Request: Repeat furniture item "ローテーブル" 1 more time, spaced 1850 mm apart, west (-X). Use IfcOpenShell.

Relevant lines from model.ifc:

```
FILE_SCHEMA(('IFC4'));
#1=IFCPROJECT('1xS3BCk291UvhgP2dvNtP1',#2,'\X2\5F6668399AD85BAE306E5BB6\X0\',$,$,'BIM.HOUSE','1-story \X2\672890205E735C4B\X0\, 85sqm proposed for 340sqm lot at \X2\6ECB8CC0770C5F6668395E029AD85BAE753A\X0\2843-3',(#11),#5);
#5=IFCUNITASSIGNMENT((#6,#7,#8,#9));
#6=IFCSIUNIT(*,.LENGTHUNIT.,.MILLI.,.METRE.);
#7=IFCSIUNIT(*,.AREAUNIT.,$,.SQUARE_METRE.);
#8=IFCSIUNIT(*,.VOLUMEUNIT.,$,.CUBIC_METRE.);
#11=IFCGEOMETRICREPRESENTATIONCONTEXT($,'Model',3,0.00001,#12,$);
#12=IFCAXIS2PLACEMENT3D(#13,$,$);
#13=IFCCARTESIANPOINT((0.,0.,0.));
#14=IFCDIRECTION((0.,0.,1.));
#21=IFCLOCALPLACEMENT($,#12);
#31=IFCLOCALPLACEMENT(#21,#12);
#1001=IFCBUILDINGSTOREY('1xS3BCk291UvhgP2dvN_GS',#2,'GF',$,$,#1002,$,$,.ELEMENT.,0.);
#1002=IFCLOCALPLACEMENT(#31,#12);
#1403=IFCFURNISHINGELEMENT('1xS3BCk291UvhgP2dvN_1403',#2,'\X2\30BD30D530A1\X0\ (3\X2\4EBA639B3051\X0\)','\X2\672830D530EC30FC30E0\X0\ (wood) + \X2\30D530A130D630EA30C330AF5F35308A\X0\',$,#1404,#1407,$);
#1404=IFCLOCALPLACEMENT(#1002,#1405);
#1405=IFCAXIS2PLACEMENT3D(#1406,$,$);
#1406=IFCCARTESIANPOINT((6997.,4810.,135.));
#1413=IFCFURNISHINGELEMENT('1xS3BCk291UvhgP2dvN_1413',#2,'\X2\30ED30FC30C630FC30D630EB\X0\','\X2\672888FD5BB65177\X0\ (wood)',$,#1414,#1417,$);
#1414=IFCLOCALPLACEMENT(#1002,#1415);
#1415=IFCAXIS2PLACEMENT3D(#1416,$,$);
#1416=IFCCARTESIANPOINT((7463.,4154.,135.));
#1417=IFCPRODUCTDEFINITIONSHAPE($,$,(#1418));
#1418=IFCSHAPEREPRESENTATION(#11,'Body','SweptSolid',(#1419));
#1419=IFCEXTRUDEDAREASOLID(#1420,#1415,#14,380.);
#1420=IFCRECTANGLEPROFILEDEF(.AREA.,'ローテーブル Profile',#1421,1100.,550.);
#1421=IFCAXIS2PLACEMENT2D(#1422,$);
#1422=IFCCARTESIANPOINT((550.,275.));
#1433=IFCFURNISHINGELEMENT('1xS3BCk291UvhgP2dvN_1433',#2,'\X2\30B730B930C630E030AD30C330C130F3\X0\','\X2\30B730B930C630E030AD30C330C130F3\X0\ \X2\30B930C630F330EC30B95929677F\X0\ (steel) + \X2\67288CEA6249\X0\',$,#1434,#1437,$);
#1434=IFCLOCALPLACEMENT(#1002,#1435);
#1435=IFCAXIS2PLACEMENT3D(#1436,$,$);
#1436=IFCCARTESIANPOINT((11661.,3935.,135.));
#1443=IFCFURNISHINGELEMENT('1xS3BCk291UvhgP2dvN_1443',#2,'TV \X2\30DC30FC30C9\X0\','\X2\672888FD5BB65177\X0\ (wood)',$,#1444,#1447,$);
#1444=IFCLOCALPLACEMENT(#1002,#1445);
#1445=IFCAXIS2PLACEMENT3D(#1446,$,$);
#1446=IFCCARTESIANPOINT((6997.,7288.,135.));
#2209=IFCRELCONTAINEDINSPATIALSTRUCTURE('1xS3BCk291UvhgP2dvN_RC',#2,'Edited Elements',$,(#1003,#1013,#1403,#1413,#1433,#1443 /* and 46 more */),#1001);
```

```python
import numpy as np
import ifcopenshell
import ifcopenshell.api.geometry
import ifcopenshell.api.root
import ifcopenshell.util.element
import ifcopenshell.util.placement

model = ifcopenshell.open("model.ifc")


def reuse_history(source, copy):
    """copy_class also copies each property set's owner history, people and application; keep the originals."""
    for rel in copy.IsDefinedBy:
        if rel.is_a("IfcRelDefinesByProperties") and (history := rel.RelatingPropertyDefinition.OwnerHistory):
            rel.RelatingPropertyDefinition.OwnerHistory = source.OwnerHistory
            ifcopenshell.util.element.remove_deep2(model, history)


source = model.by_guid("1xS3BCk291UvhgP2dvN_1413")
base = ifcopenshell.util.placement.get_local_placement(source.ObjectPlacement)
step = np.array([-1.0, 0.0, 0.0]) * 1850.0

for i in range(1, 2):
    copy = ifcopenshell.api.root.copy_class(model, product=source)
    copy.Representation = ifcopenshell.util.element.copy_deep(
        model, source.Representation, exclude=["IfcGeometricRepresentationContext", "IfcRepresentationMap"]
    )
    reuse_history(source, copy)
    matrix = base.copy()
    matrix[:3, 3] += i * step
    print("added at", matrix[:3, 3].round(3) + 0.0)
    ifcopenshell.api.geometry.edit_object_placement(model, product=copy, matrix=matrix, is_si=False)

model.write("model-out.ifc")
```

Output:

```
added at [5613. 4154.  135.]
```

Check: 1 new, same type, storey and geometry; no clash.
